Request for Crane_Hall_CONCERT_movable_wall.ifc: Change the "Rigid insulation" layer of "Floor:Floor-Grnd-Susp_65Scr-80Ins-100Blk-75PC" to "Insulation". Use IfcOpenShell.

First a look at what the model holds.

```python
import ifcopenshell
import ifcopenshell.util.element

model = ifcopenshell.open("Crane_Hall_CONCERT_movable_wall.ifc")
print(model.schema)
for layer_set in model.by_type("IfcMaterialLayerSet"):
    if layer_set.LayerSetName == "Floor:Floor-Grnd-Susp_65Scr-80Ins-100Blk-75PC":
        for layer in layer_set.MaterialLayers:
            print(layer.id(), layer.Material and layer.Material.Name, layer.LayerThickness, sep=" | ")
        print(len(ifcopenshell.util.element.get_elements_by_material(model, layer_set)), "elements and types use it")
print(sorted(m.Name for m in model.by_type("IfcMaterial") if m.Name)[:60])
```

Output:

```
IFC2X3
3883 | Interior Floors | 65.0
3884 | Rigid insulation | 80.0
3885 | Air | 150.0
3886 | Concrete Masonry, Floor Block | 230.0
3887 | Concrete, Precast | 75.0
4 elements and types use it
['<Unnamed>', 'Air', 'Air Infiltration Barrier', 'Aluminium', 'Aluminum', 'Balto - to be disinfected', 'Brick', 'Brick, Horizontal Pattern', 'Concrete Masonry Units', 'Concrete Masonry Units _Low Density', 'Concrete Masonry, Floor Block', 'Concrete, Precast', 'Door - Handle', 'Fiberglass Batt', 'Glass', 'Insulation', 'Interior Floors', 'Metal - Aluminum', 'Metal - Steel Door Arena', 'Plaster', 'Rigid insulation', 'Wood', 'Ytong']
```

```python
import ifcopenshell
import ifcopenshell.api.material

model = ifcopenshell.open("Crane_Hall_CONCERT_movable_wall.ifc")

layer_set = next(s for s in model.by_type("IfcMaterialLayerSet") if s.LayerSetName == "Floor:Floor-Grnd-Susp_65Scr-80Ins-100Blk-75PC")
layer = next(l for l in layer_set.MaterialLayers if l.Material and l.Material.Name == "Rigid insulation")
material = next(m for m in model.by_type("IfcMaterial") if m.Name == "Insulation")

# Point this one layer at the other material; renaming the old one would change it everywhere.
ifcopenshell.api.material.edit_layer(model, layer=layer, attributes={}, material=material)

print([l.Material.Name if l.Material else None for l in layer_set.MaterialLayers])

model.write("Crane_Hall_CONCERT_movable_wall_edited.ifc")
```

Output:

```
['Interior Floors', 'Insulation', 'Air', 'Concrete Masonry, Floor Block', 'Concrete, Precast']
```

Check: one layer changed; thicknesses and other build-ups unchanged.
